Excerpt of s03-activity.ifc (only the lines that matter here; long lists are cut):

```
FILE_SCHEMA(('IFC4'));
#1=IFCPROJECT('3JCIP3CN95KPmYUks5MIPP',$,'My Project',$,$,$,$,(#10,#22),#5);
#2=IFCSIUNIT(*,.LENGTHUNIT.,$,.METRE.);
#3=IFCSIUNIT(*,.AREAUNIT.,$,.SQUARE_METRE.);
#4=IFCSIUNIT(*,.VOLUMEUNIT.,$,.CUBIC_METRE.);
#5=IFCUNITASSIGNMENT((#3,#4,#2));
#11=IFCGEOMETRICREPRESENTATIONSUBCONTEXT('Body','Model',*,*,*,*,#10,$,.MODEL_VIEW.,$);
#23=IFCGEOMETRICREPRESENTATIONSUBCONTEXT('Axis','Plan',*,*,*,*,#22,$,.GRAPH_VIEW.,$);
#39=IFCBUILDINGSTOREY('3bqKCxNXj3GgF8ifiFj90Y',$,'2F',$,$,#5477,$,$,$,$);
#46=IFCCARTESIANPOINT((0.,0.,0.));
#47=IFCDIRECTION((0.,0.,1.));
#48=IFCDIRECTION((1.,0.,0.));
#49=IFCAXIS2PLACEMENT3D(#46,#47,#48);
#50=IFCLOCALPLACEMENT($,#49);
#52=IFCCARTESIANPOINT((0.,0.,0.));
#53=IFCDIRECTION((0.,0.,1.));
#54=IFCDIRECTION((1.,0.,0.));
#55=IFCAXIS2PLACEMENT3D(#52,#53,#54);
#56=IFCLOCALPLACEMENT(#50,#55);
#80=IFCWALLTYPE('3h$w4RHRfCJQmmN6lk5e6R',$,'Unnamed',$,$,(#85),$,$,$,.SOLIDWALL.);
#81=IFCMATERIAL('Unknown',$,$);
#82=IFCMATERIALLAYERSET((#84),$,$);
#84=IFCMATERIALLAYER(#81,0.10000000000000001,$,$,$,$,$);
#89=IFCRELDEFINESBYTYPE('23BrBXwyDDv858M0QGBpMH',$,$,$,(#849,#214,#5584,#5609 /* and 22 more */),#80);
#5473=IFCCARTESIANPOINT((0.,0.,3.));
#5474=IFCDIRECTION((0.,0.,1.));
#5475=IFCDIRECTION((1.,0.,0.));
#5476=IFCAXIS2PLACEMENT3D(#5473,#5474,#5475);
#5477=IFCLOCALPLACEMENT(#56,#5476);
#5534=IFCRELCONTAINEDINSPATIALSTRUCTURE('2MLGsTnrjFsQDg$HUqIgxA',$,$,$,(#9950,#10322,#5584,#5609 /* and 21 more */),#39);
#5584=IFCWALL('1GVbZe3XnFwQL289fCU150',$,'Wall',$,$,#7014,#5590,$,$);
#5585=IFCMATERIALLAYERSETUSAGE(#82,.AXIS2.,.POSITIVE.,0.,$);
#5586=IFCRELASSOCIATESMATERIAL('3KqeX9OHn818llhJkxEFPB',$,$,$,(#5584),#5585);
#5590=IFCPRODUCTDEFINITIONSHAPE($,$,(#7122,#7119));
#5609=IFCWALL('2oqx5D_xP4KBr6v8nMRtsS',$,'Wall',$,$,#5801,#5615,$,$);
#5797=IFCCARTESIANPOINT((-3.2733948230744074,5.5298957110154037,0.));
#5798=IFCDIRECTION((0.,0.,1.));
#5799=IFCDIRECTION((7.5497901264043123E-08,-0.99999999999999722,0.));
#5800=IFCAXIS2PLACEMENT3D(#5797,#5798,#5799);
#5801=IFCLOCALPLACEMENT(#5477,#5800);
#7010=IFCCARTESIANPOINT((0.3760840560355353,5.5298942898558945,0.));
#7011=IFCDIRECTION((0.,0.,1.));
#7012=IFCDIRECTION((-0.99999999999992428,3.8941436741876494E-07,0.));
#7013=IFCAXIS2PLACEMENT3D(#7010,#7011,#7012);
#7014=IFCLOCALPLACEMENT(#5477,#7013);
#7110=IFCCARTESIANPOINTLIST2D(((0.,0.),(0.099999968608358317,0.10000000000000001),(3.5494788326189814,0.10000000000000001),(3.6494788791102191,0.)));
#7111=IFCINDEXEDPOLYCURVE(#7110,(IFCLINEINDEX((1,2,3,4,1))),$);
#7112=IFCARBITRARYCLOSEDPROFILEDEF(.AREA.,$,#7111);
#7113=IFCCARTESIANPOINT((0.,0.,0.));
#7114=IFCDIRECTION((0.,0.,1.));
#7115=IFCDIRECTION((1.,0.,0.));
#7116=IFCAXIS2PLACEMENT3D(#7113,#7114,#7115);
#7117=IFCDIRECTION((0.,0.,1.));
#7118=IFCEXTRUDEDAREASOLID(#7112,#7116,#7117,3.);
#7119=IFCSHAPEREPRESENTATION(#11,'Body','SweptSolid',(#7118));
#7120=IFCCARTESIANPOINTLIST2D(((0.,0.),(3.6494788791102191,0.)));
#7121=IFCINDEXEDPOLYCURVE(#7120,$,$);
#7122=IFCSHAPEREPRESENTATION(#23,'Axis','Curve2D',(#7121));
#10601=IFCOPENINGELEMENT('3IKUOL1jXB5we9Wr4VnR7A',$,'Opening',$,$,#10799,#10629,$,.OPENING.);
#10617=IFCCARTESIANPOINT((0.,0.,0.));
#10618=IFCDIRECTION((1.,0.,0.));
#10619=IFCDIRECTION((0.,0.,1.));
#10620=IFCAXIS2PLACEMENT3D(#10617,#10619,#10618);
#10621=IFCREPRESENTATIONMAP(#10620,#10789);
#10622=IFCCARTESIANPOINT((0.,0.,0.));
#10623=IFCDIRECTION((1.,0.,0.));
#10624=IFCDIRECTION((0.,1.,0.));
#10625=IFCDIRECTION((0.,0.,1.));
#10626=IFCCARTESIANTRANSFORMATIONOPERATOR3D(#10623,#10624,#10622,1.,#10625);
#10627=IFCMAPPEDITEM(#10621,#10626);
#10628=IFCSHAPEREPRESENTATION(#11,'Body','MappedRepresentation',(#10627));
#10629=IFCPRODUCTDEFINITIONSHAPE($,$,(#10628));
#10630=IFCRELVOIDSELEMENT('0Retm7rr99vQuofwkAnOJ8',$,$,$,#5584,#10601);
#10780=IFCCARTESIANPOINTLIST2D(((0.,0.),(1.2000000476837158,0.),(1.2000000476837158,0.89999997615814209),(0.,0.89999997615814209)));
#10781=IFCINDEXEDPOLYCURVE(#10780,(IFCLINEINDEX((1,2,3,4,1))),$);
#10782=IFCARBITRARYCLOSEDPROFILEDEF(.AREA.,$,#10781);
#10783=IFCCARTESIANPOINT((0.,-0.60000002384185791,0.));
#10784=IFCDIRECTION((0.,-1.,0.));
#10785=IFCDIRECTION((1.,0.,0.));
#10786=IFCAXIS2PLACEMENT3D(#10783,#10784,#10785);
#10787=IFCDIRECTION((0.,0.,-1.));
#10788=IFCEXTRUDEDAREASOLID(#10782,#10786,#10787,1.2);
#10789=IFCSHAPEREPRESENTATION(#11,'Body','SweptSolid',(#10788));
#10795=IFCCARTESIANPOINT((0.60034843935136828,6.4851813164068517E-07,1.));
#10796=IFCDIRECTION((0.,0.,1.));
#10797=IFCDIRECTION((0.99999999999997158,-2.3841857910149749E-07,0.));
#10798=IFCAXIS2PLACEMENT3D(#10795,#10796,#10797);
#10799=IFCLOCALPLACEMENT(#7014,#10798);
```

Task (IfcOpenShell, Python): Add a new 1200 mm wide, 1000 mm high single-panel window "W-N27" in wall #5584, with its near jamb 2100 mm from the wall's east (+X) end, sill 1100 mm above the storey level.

```python
import numpy as np
import ifcopenshell
import ifcopenshell.api.feature
import ifcopenshell.api.geometry
import ifcopenshell.api.root
import ifcopenshell.api.spatial
import ifcopenshell.geom
import ifcopenshell.util.element
import ifcopenshell.util.placement
import ifcopenshell.util.representation
import ifcopenshell.util.shape
import ifcopenshell.util.unit

model = ifcopenshell.open("s03-activity.ifc")
unit_scale = ifcopenshell.util.unit.calculate_unit_scale(model)
settings = ifcopenshell.geom.settings()


def volume(element):
    """Net volume in cubic metres, openings subtracted."""
    shape = ifcopenshell.geom.create_shape(settings, element)
    return ifcopenshell.util.shape.get_volume(shape.geometry)


wall = model.by_guid("1GVbZe3XnFwQL289fCU150")
storey = ifcopenshell.util.element.get_container(wall, ifc_class="IfcBuildingStorey")
context = ifcopenshell.util.representation.get_context(model, "Model", "Body", "MODEL_VIEW")
before = volume(wall)

width, height, from_end, sill = 1.2, 1, 2.1, 1.1  # metres

# The wall runs along its own X axis, and the end named is its -X end.
wall_shape = ifcopenshell.geom.create_shape(settings, wall)
x, y, z = ifcopenshell.util.shape.get_vertices(wall_shape.geometry).T
start = x.min() + from_end
face, thickness = float(y.min()), float(y.max() - y.min())
wall_matrix = ifcopenshell.util.placement.get_local_placement(wall.ObjectPlacement)
level = ifcopenshell.util.placement.get_local_placement(storey.ObjectPlacement)[2, 3]


def in_wall(x, y):
    """Placement at x, y metres in the wall's axes, at sill height."""
    matrix = wall_matrix.copy()
    matrix[:, 3] = wall_matrix @ np.array([x / unit_scale, y / unit_scale, 0.0, 1.0])
    matrix[2, 3] = level + sill / unit_scale
    return matrix


# Opening: a box that overshoots both wall faces by 50 mm.
opening = ifcopenshell.api.root.create_entity(model, ifc_class="IfcOpeningElement", predefined_type="OPENING")
box = ifcopenshell.api.geometry.add_wall_representation(
    model, context=context, length=width, height=height, thickness=thickness + 0.1
)
ifcopenshell.api.geometry.assign_representation(model, product=opening, representation=box)
ifcopenshell.api.geometry.edit_object_placement(model, product=opening, matrix=in_wall(start, face - 0.05), is_si=False)
ifcopenshell.api.feature.add_feature(model, feature=opening, element=wall)

window = ifcopenshell.api.root.create_entity(model, ifc_class="IfcWindow", name="W-N27", predefined_type="WINDOW")
window.OverallWidth, window.OverallHeight = width / unit_scale, height / unit_scale
window.PartitioningType = "SINGLE_PANEL"
body = ifcopenshell.api.geometry.add_window_representation(
    model,
    context=context,
    overall_width=window.OverallWidth,
    overall_height=window.OverallHeight,
    partition_type="SINGLE_PANEL",
)
ifcopenshell.api.geometry.assign_representation(model, product=window, representation=body)
ifcopenshell.api.spatial.assign_container(model, products=[window], relating_structure=storey)
ifcopenshell.api.feature.add_filling(model, opening=opening, element=window)

# Centre the window in the wall's thickness.
ifcopenshell.api.geometry.edit_object_placement(model, product=window, matrix=in_wall(start, face), is_si=False)
window_shape = ifcopenshell.geom.create_shape(settings, window)
depth = ifcopenshell.util.shape.get_vertices(window_shape.geometry)[:, 1]
offset = face + thickness / 2 - (depth.min() + depth.max()) / 2
ifcopenshell.api.geometry.edit_object_placement(model, product=window, matrix=in_wall(start, offset), is_si=False)

after = volume(wall)

print(f"wall volume {before:.3f} -> {after:.3f} m3")

model.write("s03-activity_updated.ifc")
```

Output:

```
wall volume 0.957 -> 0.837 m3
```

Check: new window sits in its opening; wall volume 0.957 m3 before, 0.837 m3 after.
